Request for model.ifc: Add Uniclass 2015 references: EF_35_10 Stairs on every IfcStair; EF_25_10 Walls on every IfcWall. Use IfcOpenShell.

First a look at what the model holds.

```python
import ifcopenshell

model = ifcopenshell.open("model.ifc")
print(model.schema)
print("classifications:", [c.Name for c in model.by_type("IfcClassification")])
for ifc_class in ("IfcDoor", "IfcRoof", "IfcStair", "IfcWall", "IfcWindow"):
    print(ifc_class, len(model.by_type(ifc_class)))
```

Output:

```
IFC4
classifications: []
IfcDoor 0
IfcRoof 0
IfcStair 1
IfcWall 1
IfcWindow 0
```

```python
import ifcopenshell
import ifcopenshell.api.classification

model = ifcopenshell.open("model.ifc")

system = ifcopenshell.api.classification.add_classification(model, classification="Uniclass 2015")

codes = {
    "IfcStair": ("EF_35_10", "Stairs"),
    "IfcWall": ("EF_25_10", "Walls"),
}
for ifc_class, (code, name) in codes.items():
    products = model.by_type(ifc_class)
    ifcopenshell.api.classification.add_reference(
        model, products=products, classification=system, identification=code, name=name
    )
    print(code, len(products))

model.write("model_edited.ifc")
```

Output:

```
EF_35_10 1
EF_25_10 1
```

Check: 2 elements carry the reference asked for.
